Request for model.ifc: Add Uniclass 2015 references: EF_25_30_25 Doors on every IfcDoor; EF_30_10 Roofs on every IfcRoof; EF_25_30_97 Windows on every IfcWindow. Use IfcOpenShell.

First a look at what the model holds.

```python
import ifcopenshell

model = ifcopenshell.open("model.ifc")
print(model.schema)
print("classifications:", [c.Name for c in model.by_type("IfcClassification")])
for ifc_class in ("IfcDoor", "IfcRoof", "IfcStair", "IfcWall", "IfcWindow"):
    print(ifc_class, len(model.by_type(ifc_class)))
```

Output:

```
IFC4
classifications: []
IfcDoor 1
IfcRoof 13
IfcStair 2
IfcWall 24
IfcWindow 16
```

```python
import ifcopenshell
import ifcopenshell.api.classification

model = ifcopenshell.open("model.ifc")

system = ifcopenshell.api.classification.add_classification(model, classification="Uniclass 2015")

codes = {
    "IfcDoor": ("EF_25_30_25", "Doors"),
    "IfcRoof": ("EF_30_10", "Roofs"),
    "IfcWindow": ("EF_25_30_97", "Windows"),
}
for ifc_class, (code, name) in codes.items():
    products = model.by_type(ifc_class)
    ifcopenshell.api.classification.add_reference(
        model, products=products, classification=system, identification=code, name=name
    )
    print(code, len(products))

model.write("model_v2.ifc")
```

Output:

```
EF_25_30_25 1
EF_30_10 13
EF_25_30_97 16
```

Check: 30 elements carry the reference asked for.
